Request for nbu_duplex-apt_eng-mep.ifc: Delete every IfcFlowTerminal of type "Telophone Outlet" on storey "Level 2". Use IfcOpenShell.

First a look at what the model holds.

```python
import ifcopenshell
import ifcopenshell.util.element

model = ifcopenshell.open("nbu_duplex-apt_eng-mep.ifc")
print(model.schema)
storey = next(s for s in model.by_type("IfcBuildingStorey") if s.Name == "Level 2")
terminals = [e for e in ifcopenshell.util.element.get_decomposition(storey) if e.is_a("IfcFlowTerminal")]
seen = {}
for e in terminals:
    element_type = ifcopenshell.util.element.get_type(e)
    name = element_type.Name if element_type not in (None, e) else None
    seen[name] = seen.get(name, 0) + 1
for name, count in sorted(seen.items(), key=str):
    print(count, "x", name)
```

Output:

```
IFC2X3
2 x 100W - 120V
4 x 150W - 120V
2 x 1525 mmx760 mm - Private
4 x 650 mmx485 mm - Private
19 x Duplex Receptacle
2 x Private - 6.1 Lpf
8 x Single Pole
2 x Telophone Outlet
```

```python
import ifcopenshell
import ifcopenshell.api.root
import ifcopenshell.util.element

model = ifcopenshell.open("nbu_duplex-apt_eng-mep.ifc")

storey = next(s for s in model.by_type("IfcBuildingStorey") if s.Name == "Level 2")
terminals = [e for e in ifcopenshell.util.element.get_decomposition(storey) if e.is_a("IfcFlowTerminal")]
targets = [e for e in terminals if (t := ifcopenshell.util.element.get_type(e)) not in (None, e) and t.Name == "Telophone Outlet"]

for e in targets:
    ifcopenshell.api.root.remove_product(model, product=e)
print(len(targets), "removed")

model.write("nbu_duplex-apt_eng-mep_v2.ifc")
```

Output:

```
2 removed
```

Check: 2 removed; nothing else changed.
